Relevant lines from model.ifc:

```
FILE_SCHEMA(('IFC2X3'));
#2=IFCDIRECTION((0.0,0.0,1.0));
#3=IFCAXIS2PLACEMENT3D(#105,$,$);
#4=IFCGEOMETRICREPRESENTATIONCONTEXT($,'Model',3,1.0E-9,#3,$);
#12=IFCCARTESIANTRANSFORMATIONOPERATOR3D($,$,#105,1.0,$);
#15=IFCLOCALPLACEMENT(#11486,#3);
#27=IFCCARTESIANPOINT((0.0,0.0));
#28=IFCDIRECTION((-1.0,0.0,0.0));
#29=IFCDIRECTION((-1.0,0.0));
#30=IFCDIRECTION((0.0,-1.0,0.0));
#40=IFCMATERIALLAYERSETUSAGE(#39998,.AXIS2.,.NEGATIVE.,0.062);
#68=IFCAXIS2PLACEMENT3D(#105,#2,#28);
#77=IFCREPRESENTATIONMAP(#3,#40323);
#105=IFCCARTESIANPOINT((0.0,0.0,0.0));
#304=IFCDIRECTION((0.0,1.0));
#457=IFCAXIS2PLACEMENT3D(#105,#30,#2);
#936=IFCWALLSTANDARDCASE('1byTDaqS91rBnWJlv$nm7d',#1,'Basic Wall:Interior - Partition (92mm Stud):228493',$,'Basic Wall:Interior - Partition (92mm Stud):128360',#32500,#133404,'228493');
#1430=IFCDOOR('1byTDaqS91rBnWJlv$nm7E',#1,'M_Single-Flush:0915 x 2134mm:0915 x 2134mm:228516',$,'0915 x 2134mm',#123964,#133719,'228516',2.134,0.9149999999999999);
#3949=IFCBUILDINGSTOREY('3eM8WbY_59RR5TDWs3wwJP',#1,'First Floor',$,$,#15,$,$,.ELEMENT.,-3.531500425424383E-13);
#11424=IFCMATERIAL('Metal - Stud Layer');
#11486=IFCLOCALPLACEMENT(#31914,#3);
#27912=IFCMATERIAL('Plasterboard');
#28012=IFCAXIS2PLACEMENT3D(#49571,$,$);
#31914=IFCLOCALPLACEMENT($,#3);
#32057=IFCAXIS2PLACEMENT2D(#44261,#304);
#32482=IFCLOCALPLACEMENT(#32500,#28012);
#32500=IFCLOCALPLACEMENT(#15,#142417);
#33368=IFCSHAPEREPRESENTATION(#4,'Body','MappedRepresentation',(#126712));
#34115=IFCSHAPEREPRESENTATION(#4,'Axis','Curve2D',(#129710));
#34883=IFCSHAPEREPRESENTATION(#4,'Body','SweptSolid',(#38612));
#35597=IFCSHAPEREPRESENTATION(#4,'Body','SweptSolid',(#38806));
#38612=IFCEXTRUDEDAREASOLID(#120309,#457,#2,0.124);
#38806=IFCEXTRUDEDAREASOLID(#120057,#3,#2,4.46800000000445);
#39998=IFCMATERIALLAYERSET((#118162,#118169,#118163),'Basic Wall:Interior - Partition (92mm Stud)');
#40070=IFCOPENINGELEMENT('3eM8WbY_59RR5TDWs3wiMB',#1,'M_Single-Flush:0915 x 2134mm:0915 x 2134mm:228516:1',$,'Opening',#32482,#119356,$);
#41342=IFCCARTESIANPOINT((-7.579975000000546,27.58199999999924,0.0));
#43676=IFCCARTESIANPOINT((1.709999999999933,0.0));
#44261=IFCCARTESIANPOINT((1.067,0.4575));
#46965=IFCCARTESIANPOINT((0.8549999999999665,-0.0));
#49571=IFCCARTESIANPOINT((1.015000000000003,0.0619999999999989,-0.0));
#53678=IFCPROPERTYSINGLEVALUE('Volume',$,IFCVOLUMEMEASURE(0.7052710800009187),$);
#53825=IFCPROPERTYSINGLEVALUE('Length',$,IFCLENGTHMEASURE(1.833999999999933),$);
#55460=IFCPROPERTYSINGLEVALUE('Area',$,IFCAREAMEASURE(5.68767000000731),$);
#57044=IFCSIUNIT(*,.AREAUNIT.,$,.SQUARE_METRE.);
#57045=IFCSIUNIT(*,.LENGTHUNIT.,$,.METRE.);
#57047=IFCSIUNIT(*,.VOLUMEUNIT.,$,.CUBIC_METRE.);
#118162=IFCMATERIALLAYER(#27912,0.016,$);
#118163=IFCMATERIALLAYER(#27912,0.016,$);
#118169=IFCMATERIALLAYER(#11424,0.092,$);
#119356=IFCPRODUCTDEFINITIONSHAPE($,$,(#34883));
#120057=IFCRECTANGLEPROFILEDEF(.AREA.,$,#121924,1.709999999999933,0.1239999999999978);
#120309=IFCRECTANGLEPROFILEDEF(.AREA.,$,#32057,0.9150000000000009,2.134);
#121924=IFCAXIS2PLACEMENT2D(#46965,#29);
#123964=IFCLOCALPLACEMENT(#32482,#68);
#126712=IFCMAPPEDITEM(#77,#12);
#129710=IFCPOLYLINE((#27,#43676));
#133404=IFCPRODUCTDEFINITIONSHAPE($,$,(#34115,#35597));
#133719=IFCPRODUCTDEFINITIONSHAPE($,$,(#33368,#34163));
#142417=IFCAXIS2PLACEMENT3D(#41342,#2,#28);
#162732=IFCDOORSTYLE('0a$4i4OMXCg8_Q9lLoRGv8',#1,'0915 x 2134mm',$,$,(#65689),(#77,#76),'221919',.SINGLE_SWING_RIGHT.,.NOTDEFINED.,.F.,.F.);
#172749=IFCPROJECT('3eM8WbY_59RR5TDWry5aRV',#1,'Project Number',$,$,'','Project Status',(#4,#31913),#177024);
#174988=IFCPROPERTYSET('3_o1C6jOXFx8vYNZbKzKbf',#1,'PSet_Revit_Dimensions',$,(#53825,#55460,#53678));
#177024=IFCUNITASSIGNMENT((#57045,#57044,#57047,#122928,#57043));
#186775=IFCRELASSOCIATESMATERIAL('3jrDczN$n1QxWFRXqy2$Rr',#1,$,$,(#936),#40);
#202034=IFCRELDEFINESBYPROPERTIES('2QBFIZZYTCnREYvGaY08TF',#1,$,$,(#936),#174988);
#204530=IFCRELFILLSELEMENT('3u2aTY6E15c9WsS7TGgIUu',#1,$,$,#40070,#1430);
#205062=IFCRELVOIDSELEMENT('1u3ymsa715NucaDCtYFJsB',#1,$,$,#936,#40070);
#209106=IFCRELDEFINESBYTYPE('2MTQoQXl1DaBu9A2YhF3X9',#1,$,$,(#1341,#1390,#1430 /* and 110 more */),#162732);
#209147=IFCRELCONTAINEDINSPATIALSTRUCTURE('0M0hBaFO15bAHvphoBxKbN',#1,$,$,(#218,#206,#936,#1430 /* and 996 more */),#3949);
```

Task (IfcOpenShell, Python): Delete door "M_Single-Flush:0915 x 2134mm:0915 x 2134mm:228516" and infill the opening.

```python
import ifcopenshell
import ifcopenshell.api.feature
import ifcopenshell.api.pset
import ifcopenshell.api.root
import ifcopenshell.geom
import ifcopenshell.util.element
import ifcopenshell.util.shape
import ifcopenshell.util.unit

model = ifcopenshell.open("model.ifc")
area_scale = ifcopenshell.util.unit.calculate_unit_scale(model, "AREAUNIT")
volume_scale = ifcopenshell.util.unit.calculate_unit_scale(model, "VOLUMEUNIT")
settings = ifcopenshell.geom.settings()


def volume(element):
    """Net volume in cubic metres, openings subtracted."""
    shape = ifcopenshell.geom.create_shape(settings, element)
    return ifcopenshell.util.shape.get_volume(shape.geometry)


door = model.by_id(1430)
opening = door.FillsVoids[0].RelatingOpeningElement
wall = opening.VoidsElements[0].RelatingBuildingElement
before = volume(wall)

ifcopenshell.api.root.remove_product(model, product=door)
ifcopenshell.api.feature.remove_feature(model, feature=opening)

after = volume(wall)
thickness = 0.124  # wall thickness in metres

# Update the wall's stored quantities.
pset = model.by_id(ifcopenshell.util.element.get_pset(wall, "PSet_Revit_Dimensions", should_inherit=False)["id"])
ifcopenshell.api.pset.edit_pset(model, pset=pset, properties={
    "Area": model.create_entity("IfcAreaMeasure", after / thickness / area_scale),
    "Volume": model.create_entity("IfcVolumeMeasure", after / volume_scale),
})

print(f"wall volume {before:.3f} -> {after:.3f} m3")

model.write("model-out.ifc")
```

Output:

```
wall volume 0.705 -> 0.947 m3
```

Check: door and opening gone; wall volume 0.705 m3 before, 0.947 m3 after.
